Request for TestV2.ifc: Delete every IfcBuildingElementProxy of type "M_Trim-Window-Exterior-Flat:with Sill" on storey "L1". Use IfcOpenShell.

First a look at what the model holds.

```python
import ifcopenshell
import ifcopenshell.util.element

model = ifcopenshell.open("TestV2.ifc")
print(model.schema)
storey = next(s for s in model.by_type("IfcBuildingStorey") if s.Name == "L1")
proxies = [e for e in ifcopenshell.util.element.get_decomposition(storey) if e.is_a("IfcBuildingElementProxy")]
seen = {}
for e in proxies:
    element_type = ifcopenshell.util.element.get_type(e)
    name = element_type.Name if element_type not in (None, e) else None
    seen[name] = seen.get(name, 0) + 1
for name, count in sorted(seen.items(), key=str):
    print(count, "x", name)
```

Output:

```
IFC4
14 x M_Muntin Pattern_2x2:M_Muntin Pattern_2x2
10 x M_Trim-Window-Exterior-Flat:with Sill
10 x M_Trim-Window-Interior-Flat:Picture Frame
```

```python
import ifcopenshell
import ifcopenshell.api.root
import ifcopenshell.util.element

model = ifcopenshell.open("TestV2.ifc")

storey = next(s for s in model.by_type("IfcBuildingStorey") if s.Name == "L1")
proxies = [e for e in ifcopenshell.util.element.get_decomposition(storey) if e.is_a("IfcBuildingElementProxy")]
targets = [e for e in proxies if (t := ifcopenshell.util.element.get_type(e)) not in (None, e) and t.Name == "M_Trim-Window-Exterior-Flat:with Sill"]

for e in targets:
    ifcopenshell.api.root.remove_product(model, product=e)
print(len(targets), "removed")

model.write("TestV2_v2.ifc")
```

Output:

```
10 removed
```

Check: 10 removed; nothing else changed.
